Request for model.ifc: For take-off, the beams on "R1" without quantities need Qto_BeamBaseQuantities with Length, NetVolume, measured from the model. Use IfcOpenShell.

First a look at what the model holds.

```python
import ifcopenshell
import ifcopenshell.util.element
import ifcopenshell.util.unit

model = ifcopenshell.open("model.ifc")
print(model.schema)
for unit_type in ("LENGTHUNIT", "AREAUNIT", "VOLUMEUNIT"):
    print(unit_type, ifcopenshell.util.unit.calculate_unit_scale(model, unit_type))
storey = next(s for s in model.by_type("IfcBuildingStorey") if s.Name == "R1")
beams = [e for e in ifcopenshell.util.element.get_decomposition(storey) if e.is_a("IfcBeam")]
for e in sorted(beams, key=lambda e: e.id()):
    print(e.id(), e.is_a(), e.Name, list(ifcopenshell.util.element.get_psets(e, qtos_only=True)), sep=" | ")
```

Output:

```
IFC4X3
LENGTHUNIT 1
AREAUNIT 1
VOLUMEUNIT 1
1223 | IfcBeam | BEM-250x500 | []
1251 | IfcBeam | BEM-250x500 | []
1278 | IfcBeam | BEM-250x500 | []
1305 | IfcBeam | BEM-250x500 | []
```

```python
import ifcopenshell
import ifcopenshell.api.pset
import ifcopenshell.geom
import ifcopenshell.util.element
import ifcopenshell.util.shape
import ifcopenshell.util.unit

model = ifcopenshell.open("model.ifc")
unit_scale = ifcopenshell.util.unit.calculate_unit_scale(model)
volume_scale = ifcopenshell.util.unit.calculate_unit_scale(model, "VOLUMEUNIT")
settings = ifcopenshell.geom.settings()

storey = next(s for s in model.by_type("IfcBuildingStorey") if s.Name == "R1")
beams = [e for e in ifcopenshell.util.element.get_decomposition(storey) if e.is_a("IfcBeam")]

for e in sorted(beams, key=lambda e: e.id()):
    if ifcopenshell.util.element.get_psets(e, qtos_only=True, should_inherit=False):
        continue
    # Geometry comes back in metres, in the element's own axes.
    shape = ifcopenshell.geom.create_shape(settings, e)
    values = {
        "Length": ifcopenshell.util.shape.get_max_xyz(shape.geometry) / unit_scale,
        "NetVolume": ifcopenshell.util.shape.get_volume(shape.geometry) / volume_scale,
    }
    qto = ifcopenshell.api.pset.add_qto(model, product=e, name="Qto_BeamBaseQuantities")
    ifcopenshell.api.pset.edit_qto(model, qto=qto, properties=values)
    print(e.id(), {k: round(v, 3) for k, v in values.items()})

model.write("model_edited.ifc")
```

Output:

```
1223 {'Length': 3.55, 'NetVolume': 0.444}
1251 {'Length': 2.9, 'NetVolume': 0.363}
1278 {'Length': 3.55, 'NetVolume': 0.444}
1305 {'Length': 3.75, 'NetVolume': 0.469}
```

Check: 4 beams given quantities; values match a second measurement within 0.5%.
